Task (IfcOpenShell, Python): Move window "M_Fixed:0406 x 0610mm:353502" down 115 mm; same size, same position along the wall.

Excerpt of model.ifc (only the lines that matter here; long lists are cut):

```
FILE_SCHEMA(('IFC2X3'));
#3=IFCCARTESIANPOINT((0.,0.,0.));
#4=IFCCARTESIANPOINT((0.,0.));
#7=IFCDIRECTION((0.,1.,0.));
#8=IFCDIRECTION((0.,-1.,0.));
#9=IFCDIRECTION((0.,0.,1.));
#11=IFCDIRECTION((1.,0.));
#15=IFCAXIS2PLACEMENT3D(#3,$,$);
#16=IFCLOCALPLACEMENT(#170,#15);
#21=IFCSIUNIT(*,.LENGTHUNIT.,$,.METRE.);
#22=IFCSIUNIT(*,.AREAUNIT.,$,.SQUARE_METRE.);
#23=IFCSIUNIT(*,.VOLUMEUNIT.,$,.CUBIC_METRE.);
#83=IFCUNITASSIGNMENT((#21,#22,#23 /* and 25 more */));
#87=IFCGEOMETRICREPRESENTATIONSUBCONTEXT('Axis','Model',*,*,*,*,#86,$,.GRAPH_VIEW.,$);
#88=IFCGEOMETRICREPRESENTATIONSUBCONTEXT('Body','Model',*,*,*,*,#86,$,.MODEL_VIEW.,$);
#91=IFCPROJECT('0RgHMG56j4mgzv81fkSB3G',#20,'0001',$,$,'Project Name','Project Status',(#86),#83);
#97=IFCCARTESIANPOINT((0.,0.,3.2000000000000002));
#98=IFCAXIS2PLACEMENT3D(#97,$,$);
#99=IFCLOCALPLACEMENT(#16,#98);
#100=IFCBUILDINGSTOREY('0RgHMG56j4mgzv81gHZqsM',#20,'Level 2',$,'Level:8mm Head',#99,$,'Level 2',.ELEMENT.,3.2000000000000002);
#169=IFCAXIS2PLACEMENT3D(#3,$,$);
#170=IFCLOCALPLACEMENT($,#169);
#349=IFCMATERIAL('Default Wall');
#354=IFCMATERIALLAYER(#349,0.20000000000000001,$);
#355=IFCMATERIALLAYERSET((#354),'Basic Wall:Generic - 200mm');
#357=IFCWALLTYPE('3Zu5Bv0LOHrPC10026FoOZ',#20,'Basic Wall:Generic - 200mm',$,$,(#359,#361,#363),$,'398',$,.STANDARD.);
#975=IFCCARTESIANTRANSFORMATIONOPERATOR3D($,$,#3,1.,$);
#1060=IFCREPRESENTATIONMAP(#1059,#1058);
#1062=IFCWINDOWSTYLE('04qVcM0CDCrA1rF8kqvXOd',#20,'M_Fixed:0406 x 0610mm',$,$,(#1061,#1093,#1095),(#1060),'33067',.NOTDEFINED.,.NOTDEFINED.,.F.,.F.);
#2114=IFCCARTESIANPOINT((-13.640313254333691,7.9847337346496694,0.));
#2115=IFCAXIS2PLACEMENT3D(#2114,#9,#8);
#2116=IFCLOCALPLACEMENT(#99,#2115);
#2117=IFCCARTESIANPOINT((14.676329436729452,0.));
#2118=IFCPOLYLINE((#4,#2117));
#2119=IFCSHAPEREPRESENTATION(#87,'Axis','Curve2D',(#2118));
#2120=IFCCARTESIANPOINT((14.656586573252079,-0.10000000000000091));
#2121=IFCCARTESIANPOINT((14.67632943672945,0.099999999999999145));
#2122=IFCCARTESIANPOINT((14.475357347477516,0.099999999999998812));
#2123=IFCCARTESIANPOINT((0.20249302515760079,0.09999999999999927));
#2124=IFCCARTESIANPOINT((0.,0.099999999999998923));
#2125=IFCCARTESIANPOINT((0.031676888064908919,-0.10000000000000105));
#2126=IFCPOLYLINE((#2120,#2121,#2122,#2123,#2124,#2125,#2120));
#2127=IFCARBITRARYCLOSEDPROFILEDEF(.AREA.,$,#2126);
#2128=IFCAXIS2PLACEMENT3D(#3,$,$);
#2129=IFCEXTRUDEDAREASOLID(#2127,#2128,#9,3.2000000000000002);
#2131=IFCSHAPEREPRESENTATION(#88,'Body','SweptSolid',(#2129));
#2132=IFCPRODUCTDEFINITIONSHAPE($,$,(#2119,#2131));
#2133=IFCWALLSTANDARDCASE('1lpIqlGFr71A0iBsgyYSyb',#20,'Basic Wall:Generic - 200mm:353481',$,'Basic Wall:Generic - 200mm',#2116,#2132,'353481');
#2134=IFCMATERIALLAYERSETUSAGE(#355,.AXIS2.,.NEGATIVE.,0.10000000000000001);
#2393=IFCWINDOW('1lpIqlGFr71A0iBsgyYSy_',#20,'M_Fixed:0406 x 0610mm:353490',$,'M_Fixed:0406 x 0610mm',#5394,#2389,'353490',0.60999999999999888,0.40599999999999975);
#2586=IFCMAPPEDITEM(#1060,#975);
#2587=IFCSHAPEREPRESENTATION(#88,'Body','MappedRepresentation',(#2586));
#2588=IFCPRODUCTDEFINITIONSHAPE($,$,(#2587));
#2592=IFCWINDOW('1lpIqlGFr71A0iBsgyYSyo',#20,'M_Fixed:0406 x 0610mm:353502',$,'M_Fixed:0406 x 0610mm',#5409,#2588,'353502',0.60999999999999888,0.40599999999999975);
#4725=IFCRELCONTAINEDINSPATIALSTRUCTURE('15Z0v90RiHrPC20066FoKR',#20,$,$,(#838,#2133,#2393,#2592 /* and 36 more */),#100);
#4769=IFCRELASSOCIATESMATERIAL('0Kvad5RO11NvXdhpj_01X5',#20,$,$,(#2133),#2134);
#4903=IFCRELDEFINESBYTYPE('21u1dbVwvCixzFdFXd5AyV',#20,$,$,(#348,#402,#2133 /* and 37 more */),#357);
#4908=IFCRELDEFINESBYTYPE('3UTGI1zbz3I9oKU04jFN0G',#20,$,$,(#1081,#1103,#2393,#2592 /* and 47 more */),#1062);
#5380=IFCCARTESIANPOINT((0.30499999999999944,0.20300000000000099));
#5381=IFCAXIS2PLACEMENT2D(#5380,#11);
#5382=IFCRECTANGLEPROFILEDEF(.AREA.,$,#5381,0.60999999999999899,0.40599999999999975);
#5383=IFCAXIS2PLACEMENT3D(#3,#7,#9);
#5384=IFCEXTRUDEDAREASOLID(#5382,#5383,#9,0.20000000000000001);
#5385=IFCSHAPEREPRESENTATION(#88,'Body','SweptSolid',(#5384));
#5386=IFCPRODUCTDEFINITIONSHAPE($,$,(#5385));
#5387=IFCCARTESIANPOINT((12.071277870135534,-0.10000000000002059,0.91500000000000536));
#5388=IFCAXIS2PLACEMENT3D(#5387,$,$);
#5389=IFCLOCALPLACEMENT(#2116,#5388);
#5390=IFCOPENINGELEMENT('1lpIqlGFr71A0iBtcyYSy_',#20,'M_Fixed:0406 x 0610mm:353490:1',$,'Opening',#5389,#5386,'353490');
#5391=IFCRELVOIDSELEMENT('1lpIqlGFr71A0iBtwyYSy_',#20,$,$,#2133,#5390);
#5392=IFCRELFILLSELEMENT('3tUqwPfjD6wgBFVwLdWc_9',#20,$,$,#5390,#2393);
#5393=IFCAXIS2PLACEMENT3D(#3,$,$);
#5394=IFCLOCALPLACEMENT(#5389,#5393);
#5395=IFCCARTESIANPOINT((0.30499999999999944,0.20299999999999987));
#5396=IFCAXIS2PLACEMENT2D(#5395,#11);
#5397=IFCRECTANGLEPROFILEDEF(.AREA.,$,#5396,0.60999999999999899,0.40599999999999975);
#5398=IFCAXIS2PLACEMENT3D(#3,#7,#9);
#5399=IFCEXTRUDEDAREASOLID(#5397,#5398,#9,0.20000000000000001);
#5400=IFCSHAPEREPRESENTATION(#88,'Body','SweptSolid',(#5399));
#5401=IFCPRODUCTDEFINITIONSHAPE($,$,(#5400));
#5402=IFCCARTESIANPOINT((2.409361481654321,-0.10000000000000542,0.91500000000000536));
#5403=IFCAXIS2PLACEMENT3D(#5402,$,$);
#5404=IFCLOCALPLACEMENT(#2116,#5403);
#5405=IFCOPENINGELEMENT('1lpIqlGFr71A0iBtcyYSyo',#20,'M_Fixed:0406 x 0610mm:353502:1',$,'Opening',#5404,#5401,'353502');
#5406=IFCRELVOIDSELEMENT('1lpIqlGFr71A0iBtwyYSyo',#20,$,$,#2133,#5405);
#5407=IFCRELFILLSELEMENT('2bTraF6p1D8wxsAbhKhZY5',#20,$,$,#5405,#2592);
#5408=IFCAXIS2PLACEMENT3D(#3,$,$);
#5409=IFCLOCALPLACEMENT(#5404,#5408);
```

```python
import numpy as np
import ifcopenshell
import ifcopenshell.api.geometry
import ifcopenshell.util.placement
import ifcopenshell.util.unit

model = ifcopenshell.open("model.ifc")
unit_scale = ifcopenshell.util.unit.calculate_unit_scale(model)

window = model.by_id(2592)
opening = window.FillsVoids[0].RelatingOpeningElement
dz = -0.115 / unit_scale

shift = np.array([0.0, 0.0, dz])
# The window is placed relative to its opening, so it follows when the opening moves.
matrix = ifcopenshell.util.placement.get_local_placement(opening.ObjectPlacement)
matrix[:3, 3] += shift
ifcopenshell.api.geometry.edit_object_placement(
    model, product=opening, matrix=matrix, is_si=False, should_transform_children=True
)

print(f"moved by {dz * unit_scale:+.3f} m")

model.write("model_v2.ifc")
```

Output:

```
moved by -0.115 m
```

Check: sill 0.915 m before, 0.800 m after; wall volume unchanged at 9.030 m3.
